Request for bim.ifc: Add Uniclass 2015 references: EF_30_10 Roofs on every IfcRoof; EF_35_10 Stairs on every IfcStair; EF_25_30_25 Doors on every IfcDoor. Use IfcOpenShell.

First a look at what the model holds.

```python
import ifcopenshell

model = ifcopenshell.open("bim.ifc")
print(model.schema)
print("classifications:", [c.Name for c in model.by_type("IfcClassification")])
for ifc_class in ("IfcDoor", "IfcRoof", "IfcStair", "IfcWall", "IfcWindow"):
    print(ifc_class, len(model.by_type(ifc_class)))
```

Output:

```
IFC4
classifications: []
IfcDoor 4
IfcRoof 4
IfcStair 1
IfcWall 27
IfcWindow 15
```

```python
import ifcopenshell
import ifcopenshell.api.classification

model = ifcopenshell.open("bim.ifc")

system = ifcopenshell.api.classification.add_classification(model, classification="Uniclass 2015")

codes = {
    "IfcRoof": ("EF_30_10", "Roofs"),
    "IfcStair": ("EF_35_10", "Stairs"),
    "IfcDoor": ("EF_25_30_25", "Doors"),
}
for ifc_class, (code, name) in codes.items():
    products = model.by_type(ifc_class)
    ifcopenshell.api.classification.add_reference(
        model, products=products, classification=system, identification=code, name=name
    )
    print(code, len(products))

model.write("bim_rev.ifc")
```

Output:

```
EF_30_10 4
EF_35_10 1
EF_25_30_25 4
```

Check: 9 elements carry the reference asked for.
